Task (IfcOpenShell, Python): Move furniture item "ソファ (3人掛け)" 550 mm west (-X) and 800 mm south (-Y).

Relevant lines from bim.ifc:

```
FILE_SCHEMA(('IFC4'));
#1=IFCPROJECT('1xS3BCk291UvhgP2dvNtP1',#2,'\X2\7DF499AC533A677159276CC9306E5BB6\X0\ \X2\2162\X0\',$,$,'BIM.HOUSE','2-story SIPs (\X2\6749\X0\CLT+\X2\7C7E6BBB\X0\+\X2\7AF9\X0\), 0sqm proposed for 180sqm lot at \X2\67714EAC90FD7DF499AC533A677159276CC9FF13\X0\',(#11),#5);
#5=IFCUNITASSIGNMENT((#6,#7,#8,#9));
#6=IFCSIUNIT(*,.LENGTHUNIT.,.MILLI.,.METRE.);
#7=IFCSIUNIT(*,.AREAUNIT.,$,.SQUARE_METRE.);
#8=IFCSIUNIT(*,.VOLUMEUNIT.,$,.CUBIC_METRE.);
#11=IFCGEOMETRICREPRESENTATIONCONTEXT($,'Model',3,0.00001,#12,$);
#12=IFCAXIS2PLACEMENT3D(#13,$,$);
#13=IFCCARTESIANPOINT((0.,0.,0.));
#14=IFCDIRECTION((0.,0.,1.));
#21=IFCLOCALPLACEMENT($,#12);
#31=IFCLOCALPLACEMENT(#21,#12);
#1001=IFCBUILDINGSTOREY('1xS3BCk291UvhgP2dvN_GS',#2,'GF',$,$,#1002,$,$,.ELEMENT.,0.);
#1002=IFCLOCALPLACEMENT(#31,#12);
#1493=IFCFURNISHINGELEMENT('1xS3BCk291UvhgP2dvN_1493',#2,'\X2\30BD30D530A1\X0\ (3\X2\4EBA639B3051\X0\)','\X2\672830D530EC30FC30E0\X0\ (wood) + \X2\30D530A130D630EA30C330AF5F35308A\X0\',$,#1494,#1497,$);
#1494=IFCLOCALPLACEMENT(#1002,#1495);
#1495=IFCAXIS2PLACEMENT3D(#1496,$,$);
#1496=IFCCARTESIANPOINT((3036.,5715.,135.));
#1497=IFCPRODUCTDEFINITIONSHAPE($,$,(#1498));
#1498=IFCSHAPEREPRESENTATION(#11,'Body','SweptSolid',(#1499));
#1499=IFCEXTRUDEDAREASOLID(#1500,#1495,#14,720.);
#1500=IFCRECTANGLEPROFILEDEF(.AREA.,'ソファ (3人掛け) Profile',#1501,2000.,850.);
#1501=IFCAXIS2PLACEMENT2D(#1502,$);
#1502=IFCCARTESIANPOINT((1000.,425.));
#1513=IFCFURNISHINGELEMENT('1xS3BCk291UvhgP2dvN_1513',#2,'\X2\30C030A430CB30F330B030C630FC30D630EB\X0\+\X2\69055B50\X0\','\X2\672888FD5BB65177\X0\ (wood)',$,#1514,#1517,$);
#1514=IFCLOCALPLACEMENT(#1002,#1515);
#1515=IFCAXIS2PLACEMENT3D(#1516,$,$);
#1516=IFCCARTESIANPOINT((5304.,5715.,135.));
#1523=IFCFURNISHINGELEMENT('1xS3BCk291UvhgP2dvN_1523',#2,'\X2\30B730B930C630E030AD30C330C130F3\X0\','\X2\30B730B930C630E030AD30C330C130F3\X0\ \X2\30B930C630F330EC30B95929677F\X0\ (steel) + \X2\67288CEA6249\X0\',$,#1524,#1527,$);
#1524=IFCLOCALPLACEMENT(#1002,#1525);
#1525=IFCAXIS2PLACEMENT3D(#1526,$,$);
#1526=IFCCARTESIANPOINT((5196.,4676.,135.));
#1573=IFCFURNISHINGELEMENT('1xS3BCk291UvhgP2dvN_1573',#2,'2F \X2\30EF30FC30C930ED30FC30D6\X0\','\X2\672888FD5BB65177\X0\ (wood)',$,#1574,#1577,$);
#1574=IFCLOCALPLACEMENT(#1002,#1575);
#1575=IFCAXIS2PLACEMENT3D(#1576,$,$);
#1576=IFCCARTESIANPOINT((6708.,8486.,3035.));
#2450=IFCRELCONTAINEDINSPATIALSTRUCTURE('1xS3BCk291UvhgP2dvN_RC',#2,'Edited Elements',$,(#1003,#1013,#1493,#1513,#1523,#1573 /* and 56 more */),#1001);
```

```python
import ifcopenshell
import ifcopenshell.api.geometry
import ifcopenshell.util.placement
import ifcopenshell.util.unit

model = ifcopenshell.open("bim.ifc")
unit_scale = ifcopenshell.util.unit.calculate_unit_scale(model)

item = model.by_guid("1xS3BCk291UvhgP2dvN_1493")
matrix = ifcopenshell.util.placement.get_local_placement(item.ObjectPlacement)
matrix[0, 3] -= 0.55 / unit_scale
matrix[1, 3] -= 0.8 / unit_scale
ifcopenshell.api.geometry.edit_object_placement(model, product=item, matrix=matrix, is_si=False)

print(ifcopenshell.util.placement.get_local_placement(item.ObjectPlacement).round(3) + 0.0)

model.write("bim_rev.ifc")
```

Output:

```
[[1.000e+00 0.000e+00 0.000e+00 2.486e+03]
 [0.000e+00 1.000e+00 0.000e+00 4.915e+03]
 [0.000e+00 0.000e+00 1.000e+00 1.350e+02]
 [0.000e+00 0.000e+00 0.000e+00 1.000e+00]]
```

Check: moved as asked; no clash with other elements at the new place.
